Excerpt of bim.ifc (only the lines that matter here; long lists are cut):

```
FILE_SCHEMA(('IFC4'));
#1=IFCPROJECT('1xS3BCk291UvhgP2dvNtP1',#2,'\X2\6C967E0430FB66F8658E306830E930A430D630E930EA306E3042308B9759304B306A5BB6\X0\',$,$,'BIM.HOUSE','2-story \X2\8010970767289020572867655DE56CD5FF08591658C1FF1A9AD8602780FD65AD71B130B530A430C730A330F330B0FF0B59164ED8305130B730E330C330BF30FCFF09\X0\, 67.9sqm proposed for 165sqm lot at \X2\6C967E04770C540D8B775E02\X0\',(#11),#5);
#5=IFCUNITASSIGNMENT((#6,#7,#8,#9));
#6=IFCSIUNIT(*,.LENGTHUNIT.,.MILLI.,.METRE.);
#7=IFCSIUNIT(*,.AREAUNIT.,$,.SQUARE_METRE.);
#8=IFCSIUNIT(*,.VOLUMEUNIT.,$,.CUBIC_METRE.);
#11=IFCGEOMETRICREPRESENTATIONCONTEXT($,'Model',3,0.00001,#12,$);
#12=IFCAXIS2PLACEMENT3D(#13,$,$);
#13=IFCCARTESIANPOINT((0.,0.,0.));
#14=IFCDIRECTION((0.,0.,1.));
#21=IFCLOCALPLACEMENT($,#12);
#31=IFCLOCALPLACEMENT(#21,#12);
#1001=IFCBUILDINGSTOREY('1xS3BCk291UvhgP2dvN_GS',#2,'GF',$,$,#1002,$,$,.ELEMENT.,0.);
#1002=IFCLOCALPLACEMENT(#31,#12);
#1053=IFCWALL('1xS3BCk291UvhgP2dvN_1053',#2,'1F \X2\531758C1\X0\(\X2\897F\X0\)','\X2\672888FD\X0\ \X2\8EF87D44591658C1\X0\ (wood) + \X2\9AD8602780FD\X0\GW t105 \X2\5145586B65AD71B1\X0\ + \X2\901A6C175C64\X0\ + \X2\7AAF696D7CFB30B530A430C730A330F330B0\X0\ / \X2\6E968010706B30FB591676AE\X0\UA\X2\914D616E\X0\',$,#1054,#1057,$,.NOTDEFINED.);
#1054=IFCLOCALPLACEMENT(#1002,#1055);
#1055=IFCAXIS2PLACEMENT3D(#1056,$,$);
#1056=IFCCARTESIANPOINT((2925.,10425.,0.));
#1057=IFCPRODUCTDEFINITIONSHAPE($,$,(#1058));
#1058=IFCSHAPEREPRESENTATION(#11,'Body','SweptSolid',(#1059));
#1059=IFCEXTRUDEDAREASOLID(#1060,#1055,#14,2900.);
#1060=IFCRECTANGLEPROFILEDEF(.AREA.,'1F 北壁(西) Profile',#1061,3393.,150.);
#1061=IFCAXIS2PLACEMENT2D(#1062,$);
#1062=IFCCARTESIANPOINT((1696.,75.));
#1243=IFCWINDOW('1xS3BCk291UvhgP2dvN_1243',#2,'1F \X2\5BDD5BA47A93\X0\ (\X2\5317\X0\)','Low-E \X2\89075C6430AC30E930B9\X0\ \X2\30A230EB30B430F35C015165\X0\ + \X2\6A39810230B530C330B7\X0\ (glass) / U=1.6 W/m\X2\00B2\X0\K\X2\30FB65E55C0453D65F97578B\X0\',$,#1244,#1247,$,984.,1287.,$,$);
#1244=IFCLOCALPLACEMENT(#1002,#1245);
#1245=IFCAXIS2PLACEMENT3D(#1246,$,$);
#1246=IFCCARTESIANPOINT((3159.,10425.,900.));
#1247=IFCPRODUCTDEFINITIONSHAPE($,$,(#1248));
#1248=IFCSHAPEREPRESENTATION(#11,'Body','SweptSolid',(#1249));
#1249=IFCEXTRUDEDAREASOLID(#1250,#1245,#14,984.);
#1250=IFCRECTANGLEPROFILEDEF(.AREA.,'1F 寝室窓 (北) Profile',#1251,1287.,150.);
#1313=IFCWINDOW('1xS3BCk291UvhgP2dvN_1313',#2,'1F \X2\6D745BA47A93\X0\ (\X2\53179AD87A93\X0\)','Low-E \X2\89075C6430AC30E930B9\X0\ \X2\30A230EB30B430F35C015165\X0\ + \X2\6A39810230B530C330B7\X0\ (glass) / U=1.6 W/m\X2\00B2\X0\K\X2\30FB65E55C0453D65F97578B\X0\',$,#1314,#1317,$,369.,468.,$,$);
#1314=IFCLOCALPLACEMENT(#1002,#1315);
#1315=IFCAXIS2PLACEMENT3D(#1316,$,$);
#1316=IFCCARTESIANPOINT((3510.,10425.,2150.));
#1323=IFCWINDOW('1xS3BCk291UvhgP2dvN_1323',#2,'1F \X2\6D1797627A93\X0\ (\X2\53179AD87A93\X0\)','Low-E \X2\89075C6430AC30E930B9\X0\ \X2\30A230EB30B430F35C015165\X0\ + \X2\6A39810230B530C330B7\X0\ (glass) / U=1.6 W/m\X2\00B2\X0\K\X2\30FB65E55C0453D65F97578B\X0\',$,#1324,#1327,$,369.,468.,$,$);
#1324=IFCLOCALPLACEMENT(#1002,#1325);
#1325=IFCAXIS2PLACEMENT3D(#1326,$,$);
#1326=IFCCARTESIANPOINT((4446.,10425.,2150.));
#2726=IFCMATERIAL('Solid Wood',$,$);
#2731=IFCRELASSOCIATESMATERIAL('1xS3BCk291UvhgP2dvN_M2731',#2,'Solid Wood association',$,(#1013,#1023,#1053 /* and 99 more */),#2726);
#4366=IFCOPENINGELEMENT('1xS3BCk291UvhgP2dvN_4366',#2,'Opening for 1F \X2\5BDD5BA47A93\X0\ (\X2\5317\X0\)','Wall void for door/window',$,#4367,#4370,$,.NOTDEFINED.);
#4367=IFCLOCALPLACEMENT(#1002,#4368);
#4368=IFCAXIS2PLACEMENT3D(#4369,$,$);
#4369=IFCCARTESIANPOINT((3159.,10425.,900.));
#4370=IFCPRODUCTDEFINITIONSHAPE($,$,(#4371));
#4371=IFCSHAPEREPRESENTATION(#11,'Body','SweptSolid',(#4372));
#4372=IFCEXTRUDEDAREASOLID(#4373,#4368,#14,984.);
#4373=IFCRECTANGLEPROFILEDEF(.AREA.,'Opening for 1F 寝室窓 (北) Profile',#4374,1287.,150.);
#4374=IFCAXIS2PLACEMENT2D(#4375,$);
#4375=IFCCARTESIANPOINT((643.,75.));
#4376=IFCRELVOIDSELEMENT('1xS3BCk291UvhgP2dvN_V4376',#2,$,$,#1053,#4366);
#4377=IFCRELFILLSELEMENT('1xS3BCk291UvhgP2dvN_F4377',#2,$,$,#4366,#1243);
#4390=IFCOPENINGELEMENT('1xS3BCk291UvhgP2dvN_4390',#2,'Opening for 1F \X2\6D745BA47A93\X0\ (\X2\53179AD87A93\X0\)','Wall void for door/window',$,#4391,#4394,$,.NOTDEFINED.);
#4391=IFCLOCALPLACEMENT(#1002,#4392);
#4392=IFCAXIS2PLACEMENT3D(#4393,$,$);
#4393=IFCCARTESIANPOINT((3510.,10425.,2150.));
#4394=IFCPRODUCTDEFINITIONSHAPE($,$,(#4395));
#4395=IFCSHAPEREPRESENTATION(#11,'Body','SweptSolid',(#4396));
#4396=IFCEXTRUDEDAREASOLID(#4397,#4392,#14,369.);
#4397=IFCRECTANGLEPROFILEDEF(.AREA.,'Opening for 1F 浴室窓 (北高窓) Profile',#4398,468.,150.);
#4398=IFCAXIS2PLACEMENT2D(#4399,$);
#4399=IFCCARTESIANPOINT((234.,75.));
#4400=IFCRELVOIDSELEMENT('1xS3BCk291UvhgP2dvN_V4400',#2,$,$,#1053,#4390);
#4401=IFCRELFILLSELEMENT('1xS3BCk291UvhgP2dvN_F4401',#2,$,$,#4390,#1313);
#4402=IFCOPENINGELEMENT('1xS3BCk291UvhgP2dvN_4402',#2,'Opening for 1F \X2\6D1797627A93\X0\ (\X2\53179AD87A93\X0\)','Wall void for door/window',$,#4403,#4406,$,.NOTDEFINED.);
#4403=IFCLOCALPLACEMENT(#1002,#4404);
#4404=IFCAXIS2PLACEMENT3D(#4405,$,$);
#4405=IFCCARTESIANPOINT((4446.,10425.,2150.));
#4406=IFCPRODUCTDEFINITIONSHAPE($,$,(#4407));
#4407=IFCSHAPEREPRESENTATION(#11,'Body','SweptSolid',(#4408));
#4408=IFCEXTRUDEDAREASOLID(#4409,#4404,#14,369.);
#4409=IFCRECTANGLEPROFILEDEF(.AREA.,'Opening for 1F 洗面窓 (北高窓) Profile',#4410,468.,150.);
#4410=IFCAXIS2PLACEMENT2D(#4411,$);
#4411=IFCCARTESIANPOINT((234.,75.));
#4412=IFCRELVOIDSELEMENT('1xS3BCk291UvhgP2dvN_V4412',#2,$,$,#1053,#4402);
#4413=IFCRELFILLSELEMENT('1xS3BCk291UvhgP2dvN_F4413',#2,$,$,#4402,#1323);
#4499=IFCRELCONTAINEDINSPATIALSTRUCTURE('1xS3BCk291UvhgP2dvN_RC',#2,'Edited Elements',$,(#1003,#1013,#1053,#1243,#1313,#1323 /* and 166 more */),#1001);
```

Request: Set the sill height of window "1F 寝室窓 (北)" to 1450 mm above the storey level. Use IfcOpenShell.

```python
import numpy as np
import ifcopenshell
import ifcopenshell.api.geometry
import ifcopenshell.geom
import ifcopenshell.util.element
import ifcopenshell.util.placement
import ifcopenshell.util.shape
import ifcopenshell.util.unit

model = ifcopenshell.open("bim.ifc")
unit_scale = ifcopenshell.util.unit.calculate_unit_scale(model)

window = model.by_guid("1xS3BCk291UvhgP2dvN_1243")
opening = window.FillsVoids[0].RelatingOpeningElement
storey = ifcopenshell.util.element.get_container(window, ifc_class="IfcBuildingStorey")
level = ifcopenshell.util.placement.get_local_placement(storey.ObjectPlacement)[2, 3]

# The opening's origin need not be at the sill, so measure its lowest point.
shape = ifcopenshell.geom.create_shape(ifcopenshell.geom.settings(), opening)
bottom = ifcopenshell.util.shape.get_shape_bottom_elevation(shape, shape.geometry) / unit_scale
dz = level + 1.45 / unit_scale - bottom

shift = np.array([0.0, 0.0, dz])
# The window is not placed relative to its opening, so move both.
for product in (opening, window):
    matrix = ifcopenshell.util.placement.get_local_placement(product.ObjectPlacement)
    matrix[:3, 3] += shift
    ifcopenshell.api.geometry.edit_object_placement(model, product=product, matrix=matrix, is_si=False)

print(f"moved by {dz * unit_scale:+.3f} m")

model.write("bim_updated.ifc")
```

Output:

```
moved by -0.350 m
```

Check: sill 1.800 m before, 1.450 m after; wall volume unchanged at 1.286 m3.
